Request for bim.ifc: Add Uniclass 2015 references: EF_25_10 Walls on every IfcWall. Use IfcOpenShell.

First a look at what the model holds.

```python
import ifcopenshell

model = ifcopenshell.open("bim.ifc")
print(model.schema)
print("classifications:", [c.Name for c in model.by_type("IfcClassification")])
for ifc_class in ("IfcDoor", "IfcRoof", "IfcStair", "IfcWall", "IfcWindow"):
    print(ifc_class, len(model.by_type(ifc_class)))
```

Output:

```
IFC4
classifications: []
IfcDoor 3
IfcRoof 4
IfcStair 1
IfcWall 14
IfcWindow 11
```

```python
import ifcopenshell
import ifcopenshell.api.classification

model = ifcopenshell.open("bim.ifc")

system = ifcopenshell.api.classification.add_classification(model, classification="Uniclass 2015")

codes = {
    "IfcWall": ("EF_25_10", "Walls"),
}
for ifc_class, (code, name) in codes.items():
    products = model.by_type(ifc_class)
    ifcopenshell.api.classification.add_reference(
        model, products=products, classification=system, identification=code, name=name
    )
    print(code, len(products))

model.write("bim-out.ifc")
```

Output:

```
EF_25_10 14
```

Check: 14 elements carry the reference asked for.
